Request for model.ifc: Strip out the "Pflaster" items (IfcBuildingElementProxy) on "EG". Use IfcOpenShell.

First a look at what the model holds.

```python
import ifcopenshell
import ifcopenshell.util.element

model = ifcopenshell.open("model.ifc")
print(model.schema)
storey = next(s for s in model.by_type("IfcBuildingStorey") if s.Name == "EG")
proxies = [e for e in ifcopenshell.util.element.get_decomposition(storey) if e.is_a("IfcBuildingElementProxy")]
seen = {}
for e in proxies:
    element_type = ifcopenshell.util.element.get_type(e)
    name = element_type.Name if element_type not in (None, e) else None
    seen[name] = seen.get(name, 0) + 1
for name, count in sorted(seen.items(), key=str):
    print(count, "x", name)
```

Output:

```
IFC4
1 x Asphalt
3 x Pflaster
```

```python
import ifcopenshell
import ifcopenshell.api.root
import ifcopenshell.util.element

model = ifcopenshell.open("model.ifc")

storey = next(s for s in model.by_type("IfcBuildingStorey") if s.Name == "EG")
proxies = [e for e in ifcopenshell.util.element.get_decomposition(storey) if e.is_a("IfcBuildingElementProxy")]
targets = [e for e in proxies if (t := ifcopenshell.util.element.get_type(e)) not in (None, e) and t.Name == "Pflaster"]

for e in targets:
    ifcopenshell.api.root.remove_product(model, product=e)
print(len(targets), "removed")

model.write("model-out.ifc")
```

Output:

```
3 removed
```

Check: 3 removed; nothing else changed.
